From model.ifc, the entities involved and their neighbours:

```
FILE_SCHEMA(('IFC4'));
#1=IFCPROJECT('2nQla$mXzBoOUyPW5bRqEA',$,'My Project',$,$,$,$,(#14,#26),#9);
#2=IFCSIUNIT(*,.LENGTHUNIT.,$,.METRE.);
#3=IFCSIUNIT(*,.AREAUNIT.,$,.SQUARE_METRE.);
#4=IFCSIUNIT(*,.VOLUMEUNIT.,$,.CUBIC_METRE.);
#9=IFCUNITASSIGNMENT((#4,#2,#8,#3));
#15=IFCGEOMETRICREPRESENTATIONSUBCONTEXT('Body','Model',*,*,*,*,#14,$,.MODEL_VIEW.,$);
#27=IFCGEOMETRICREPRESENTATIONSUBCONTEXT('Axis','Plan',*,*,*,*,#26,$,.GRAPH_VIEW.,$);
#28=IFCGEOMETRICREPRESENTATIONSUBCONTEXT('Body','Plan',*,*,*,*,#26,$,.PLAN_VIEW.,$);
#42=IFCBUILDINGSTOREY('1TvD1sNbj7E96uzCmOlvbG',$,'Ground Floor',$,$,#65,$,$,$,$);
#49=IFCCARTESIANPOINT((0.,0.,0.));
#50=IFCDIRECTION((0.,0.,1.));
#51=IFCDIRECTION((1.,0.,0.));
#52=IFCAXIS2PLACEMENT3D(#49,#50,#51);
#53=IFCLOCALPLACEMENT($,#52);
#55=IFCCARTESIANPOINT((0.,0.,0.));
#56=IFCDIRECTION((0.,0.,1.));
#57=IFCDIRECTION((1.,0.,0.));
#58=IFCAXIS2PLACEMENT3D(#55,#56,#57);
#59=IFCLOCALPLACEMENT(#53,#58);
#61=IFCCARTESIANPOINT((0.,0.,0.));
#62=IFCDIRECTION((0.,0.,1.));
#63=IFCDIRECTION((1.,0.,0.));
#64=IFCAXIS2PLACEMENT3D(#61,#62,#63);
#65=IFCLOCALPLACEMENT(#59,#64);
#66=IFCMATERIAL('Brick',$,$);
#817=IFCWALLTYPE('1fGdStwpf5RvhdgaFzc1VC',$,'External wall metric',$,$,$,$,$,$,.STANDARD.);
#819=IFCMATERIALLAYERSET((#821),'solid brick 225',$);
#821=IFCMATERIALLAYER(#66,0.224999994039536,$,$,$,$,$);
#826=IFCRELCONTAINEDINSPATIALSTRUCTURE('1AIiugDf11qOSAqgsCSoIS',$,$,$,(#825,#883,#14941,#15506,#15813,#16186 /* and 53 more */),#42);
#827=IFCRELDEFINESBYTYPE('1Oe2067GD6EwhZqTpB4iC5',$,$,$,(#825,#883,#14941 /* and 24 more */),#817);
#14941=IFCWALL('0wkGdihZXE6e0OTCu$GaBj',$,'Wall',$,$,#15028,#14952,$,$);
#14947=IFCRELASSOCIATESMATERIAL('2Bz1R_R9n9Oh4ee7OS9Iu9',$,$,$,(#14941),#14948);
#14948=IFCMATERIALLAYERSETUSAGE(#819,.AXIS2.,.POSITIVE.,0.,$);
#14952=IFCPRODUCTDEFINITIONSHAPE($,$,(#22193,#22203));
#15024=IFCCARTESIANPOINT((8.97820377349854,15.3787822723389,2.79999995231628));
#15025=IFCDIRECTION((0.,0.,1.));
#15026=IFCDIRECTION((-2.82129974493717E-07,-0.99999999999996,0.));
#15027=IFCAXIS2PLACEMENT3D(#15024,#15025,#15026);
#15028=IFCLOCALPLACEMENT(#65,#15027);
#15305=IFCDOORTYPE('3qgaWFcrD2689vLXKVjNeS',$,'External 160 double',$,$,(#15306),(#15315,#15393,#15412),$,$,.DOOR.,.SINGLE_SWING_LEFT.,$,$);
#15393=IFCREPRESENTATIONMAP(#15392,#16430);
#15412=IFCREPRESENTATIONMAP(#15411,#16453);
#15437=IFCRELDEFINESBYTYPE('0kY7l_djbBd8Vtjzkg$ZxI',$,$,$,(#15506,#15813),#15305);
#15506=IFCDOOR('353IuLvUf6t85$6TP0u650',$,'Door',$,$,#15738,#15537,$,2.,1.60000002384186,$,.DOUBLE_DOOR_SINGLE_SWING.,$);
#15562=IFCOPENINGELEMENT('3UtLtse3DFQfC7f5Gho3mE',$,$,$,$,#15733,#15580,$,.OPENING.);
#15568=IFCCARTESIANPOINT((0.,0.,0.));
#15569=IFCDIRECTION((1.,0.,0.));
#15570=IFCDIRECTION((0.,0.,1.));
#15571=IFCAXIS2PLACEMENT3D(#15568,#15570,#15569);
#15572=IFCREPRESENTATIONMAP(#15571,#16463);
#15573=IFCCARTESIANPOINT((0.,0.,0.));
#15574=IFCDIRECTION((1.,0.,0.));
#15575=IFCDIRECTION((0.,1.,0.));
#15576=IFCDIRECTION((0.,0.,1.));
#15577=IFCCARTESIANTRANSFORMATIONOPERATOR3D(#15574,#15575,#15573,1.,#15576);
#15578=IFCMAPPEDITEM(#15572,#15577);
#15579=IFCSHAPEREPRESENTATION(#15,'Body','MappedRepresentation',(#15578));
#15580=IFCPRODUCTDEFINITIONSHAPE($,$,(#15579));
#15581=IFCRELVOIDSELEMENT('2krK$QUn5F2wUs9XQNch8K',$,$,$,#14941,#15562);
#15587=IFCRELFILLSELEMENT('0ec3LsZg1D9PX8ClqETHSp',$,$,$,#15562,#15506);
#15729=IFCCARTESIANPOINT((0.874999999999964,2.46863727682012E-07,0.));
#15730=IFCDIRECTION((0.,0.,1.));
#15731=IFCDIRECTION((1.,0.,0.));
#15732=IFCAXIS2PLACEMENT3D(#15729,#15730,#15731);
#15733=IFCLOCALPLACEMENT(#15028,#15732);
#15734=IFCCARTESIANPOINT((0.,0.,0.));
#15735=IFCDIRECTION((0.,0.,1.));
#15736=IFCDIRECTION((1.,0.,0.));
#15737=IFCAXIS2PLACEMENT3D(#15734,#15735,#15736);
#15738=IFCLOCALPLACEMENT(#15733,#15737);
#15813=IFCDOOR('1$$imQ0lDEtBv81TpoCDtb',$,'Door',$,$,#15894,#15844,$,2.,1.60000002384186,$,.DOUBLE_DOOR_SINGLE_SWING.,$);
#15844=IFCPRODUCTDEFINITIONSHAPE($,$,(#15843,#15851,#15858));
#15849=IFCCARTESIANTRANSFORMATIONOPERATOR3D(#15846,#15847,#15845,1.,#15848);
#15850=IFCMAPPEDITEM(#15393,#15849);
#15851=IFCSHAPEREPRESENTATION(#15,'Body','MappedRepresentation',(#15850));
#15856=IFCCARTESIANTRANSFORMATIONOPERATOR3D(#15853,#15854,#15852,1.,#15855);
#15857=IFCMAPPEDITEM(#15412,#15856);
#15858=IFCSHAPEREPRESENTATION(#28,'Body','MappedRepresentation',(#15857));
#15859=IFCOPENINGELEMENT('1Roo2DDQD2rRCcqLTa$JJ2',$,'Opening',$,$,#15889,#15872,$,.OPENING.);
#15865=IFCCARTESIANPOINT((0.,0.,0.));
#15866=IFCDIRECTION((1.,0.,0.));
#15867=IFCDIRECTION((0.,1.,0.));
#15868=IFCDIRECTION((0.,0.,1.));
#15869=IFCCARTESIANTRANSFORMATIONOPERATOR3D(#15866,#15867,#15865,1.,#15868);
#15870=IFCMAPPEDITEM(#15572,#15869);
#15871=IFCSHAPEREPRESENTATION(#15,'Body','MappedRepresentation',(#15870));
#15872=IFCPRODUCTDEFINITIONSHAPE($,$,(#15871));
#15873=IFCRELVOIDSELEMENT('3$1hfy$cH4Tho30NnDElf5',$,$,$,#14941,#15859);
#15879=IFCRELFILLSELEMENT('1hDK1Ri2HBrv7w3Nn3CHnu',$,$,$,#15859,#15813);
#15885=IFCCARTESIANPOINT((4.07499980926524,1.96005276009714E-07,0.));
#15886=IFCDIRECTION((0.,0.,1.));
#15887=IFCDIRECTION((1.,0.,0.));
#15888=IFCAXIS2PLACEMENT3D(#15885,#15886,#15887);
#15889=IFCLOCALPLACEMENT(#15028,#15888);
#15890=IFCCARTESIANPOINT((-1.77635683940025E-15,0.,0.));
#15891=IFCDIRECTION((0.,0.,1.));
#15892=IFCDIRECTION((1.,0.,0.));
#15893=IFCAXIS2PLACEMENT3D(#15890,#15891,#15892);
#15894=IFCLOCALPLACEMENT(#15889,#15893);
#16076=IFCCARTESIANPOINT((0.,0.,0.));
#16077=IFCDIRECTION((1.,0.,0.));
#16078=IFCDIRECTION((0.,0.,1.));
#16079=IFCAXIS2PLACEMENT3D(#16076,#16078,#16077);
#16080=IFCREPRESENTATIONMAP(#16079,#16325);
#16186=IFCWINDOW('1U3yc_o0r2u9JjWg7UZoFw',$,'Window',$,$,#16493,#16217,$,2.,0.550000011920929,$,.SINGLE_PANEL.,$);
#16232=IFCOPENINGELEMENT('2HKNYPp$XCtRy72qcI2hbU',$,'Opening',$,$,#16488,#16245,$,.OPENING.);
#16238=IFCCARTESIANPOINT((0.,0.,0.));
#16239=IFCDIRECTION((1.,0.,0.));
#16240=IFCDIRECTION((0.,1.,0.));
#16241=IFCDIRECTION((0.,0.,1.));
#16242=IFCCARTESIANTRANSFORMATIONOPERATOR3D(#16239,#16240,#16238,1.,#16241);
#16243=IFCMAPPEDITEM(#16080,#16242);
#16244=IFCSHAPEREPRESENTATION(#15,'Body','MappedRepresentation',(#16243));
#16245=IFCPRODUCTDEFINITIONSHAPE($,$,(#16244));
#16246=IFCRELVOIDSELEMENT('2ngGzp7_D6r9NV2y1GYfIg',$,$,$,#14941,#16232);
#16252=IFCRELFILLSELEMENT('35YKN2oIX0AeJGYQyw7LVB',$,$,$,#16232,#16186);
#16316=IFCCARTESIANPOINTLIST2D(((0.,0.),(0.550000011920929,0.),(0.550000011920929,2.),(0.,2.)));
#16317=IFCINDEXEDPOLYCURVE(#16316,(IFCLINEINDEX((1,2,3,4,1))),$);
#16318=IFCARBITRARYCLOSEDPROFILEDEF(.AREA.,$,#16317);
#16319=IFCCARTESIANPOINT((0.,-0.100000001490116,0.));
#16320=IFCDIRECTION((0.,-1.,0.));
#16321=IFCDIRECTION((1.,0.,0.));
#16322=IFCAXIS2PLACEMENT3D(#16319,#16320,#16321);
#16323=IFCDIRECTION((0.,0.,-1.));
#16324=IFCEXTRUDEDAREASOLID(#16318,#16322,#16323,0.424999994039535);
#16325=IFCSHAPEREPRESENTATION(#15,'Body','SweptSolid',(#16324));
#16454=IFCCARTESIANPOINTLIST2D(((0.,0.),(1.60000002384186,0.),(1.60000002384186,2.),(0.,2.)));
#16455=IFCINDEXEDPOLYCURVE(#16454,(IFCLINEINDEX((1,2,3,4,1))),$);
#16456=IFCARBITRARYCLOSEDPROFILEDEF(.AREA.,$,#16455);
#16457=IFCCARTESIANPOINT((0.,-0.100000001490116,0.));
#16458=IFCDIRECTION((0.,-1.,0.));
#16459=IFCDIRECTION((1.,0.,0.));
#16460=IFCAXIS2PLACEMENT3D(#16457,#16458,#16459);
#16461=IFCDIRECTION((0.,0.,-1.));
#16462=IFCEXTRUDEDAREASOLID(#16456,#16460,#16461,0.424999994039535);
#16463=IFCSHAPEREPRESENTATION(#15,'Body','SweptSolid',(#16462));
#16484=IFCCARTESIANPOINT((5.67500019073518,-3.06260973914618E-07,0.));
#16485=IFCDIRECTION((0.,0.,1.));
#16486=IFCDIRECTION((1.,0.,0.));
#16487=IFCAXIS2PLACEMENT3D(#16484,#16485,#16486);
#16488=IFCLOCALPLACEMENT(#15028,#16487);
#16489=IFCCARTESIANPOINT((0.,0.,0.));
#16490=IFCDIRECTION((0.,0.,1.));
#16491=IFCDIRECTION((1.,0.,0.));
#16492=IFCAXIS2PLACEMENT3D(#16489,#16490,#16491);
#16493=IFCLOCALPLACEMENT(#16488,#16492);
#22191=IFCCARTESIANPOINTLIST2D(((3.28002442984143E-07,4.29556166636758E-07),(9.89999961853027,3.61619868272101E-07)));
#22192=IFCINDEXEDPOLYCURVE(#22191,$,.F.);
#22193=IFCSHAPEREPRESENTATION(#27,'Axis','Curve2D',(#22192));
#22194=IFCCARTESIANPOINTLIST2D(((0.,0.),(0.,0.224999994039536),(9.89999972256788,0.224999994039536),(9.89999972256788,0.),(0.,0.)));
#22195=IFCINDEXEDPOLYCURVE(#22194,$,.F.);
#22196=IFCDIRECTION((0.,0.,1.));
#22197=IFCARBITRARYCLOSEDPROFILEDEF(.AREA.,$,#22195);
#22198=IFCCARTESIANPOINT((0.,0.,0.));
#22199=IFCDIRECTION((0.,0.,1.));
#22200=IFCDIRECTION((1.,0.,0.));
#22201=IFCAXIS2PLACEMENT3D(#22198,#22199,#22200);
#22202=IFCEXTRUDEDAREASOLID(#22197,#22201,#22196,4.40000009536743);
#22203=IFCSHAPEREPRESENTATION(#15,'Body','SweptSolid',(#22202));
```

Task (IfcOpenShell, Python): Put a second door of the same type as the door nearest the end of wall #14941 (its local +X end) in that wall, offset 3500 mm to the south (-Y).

```python
import ifcopenshell
import ifcopenshell.api.feature
import ifcopenshell.api.geometry
import ifcopenshell.api.root
import ifcopenshell.geom
import ifcopenshell.util.element
import ifcopenshell.util.placement
import ifcopenshell.util.shape
import ifcopenshell.util.unit

model = ifcopenshell.open("model.ifc")
unit_scale = ifcopenshell.util.unit.calculate_unit_scale(model)
settings = ifcopenshell.geom.settings()


def volume(element):
    """Net volume in cubic metres, openings subtracted."""
    shape = ifcopenshell.geom.create_shape(settings, element)
    return ifcopenshell.util.shape.get_volume(shape.geometry)


door = model.by_guid("1$$imQ0lDEtBv81TpoCDtb")
opening = door.FillsVoids[0].RelatingOpeningElement
wall = opening.VoidsElements[0].RelatingBuildingElement
before = volume(wall)
shift = ifcopenshell.util.placement.get_local_placement(wall.ObjectPlacement)[:3, 0] * 3.5 / unit_scale

# copy_class copies the void relationship, type, container and properties, but no geometry.
new_opening = ifcopenshell.api.root.copy_class(model, product=opening)
new_opening.Representation = ifcopenshell.util.element.copy_deep(
    model, opening.Representation, exclude=["IfcGeometricRepresentationContext", "IfcRepresentationMap"]
)
new_door = ifcopenshell.api.root.copy_class(model, product=door)
new_door.Representation = ifcopenshell.util.element.copy_deep(
    model, door.Representation, exclude=["IfcGeometricRepresentationContext", "IfcRepresentationMap"]
)
ifcopenshell.api.feature.add_filling(model, opening=new_opening, element=new_door)

for old, new in ((opening, new_opening), (door, new_door)):
    matrix = ifcopenshell.util.placement.get_local_placement(old.ObjectPlacement)
    matrix[:3, 3] += shift
    ifcopenshell.api.geometry.edit_object_placement(model, product=new, matrix=matrix, is_si=False)

after = volume(wall)

print(f"wall volume {before:.3f} -> {after:.3f} m3")

model.write("model_v2.ifc")
```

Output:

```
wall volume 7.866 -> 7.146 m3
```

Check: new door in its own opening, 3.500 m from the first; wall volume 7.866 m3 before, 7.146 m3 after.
